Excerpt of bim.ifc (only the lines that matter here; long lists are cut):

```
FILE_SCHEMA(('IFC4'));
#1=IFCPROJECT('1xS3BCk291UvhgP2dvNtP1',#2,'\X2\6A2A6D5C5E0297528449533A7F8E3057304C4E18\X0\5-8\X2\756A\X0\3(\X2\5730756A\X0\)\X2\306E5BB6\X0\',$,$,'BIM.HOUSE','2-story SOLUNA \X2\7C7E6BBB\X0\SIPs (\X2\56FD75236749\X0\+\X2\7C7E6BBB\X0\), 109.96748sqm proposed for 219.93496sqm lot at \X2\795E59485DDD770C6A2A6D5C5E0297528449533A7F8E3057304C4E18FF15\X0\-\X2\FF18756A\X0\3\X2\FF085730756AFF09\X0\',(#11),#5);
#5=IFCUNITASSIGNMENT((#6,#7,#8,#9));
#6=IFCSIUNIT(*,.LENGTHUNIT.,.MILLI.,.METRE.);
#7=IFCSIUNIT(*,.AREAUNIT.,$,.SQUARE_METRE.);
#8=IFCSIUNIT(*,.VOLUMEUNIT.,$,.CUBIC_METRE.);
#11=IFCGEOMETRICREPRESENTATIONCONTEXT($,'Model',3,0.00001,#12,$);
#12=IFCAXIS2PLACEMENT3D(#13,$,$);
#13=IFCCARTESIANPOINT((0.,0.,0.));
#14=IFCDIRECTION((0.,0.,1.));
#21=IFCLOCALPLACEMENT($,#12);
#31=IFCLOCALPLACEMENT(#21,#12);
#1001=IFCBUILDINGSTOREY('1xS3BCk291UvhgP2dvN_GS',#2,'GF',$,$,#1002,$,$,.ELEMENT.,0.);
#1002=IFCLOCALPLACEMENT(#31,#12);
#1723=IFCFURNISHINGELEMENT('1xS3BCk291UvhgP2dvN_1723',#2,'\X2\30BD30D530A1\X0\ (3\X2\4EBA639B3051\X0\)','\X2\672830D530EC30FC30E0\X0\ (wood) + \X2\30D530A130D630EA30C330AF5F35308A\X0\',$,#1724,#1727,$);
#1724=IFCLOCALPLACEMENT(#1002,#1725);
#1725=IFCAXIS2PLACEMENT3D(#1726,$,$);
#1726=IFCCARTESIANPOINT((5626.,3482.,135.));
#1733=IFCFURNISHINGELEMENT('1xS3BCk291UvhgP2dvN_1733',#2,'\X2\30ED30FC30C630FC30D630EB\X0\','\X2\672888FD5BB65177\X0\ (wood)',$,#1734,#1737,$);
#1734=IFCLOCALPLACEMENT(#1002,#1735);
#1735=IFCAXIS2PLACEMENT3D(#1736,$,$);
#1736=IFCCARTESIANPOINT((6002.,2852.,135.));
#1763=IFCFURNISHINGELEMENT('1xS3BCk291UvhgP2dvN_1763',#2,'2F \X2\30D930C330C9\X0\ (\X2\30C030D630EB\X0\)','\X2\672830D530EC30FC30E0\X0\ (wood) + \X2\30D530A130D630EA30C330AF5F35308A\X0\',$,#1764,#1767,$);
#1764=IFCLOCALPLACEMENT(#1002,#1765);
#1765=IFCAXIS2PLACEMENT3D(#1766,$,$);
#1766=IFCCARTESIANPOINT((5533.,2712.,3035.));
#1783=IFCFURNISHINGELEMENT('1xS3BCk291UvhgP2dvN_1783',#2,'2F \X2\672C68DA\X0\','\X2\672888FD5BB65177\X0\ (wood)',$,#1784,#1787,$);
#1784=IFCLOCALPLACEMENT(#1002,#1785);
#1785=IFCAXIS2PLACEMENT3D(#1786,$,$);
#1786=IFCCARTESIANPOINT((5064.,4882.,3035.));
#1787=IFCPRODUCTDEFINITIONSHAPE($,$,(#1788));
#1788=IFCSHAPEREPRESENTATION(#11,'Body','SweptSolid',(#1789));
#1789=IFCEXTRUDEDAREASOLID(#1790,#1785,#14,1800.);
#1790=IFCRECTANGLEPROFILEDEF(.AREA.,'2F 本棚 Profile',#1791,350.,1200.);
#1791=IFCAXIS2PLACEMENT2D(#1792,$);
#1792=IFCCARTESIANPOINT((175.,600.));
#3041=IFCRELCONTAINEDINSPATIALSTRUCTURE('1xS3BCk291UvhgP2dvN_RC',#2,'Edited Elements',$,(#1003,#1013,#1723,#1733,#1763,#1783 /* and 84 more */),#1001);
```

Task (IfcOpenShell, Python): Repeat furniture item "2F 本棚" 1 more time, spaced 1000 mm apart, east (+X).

```python
import numpy as np
import ifcopenshell
import ifcopenshell.api.geometry
import ifcopenshell.api.root
import ifcopenshell.util.element
import ifcopenshell.util.placement
import ifcopenshell.util.unit

model = ifcopenshell.open("bim.ifc")
unit_scale = ifcopenshell.util.unit.calculate_unit_scale(model)


def reuse_history(source, copy):
    """copy_class also copies each property set's owner history, people and application; keep the originals."""
    for rel in copy.IsDefinedBy:
        if rel.is_a("IfcRelDefinesByProperties") and (history := rel.RelatingPropertyDefinition.OwnerHistory):
            rel.RelatingPropertyDefinition.OwnerHistory = source.OwnerHistory
            ifcopenshell.util.element.remove_deep2(model, history)


source = model.by_guid("1xS3BCk291UvhgP2dvN_1783")
base = ifcopenshell.util.placement.get_local_placement(source.ObjectPlacement)
step = np.array([1.0, 0.0, 0.0]) * 1 / unit_scale

for i in range(1, 2):
    copy = ifcopenshell.api.root.copy_class(model, product=source)
    copy.Representation = ifcopenshell.util.element.copy_deep(
        model, source.Representation, exclude=["IfcGeometricRepresentationContext", "IfcRepresentationMap"]
    )
    reuse_history(source, copy)
    matrix = base.copy()
    matrix[:3, 3] += i * step
    print("added at", matrix[:3, 3].round(3) + 0.0)
    ifcopenshell.api.geometry.edit_object_placement(model, product=copy, matrix=matrix, is_si=False)

model.write("bim_edited.ifc")
```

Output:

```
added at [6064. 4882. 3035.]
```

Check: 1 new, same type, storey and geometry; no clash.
